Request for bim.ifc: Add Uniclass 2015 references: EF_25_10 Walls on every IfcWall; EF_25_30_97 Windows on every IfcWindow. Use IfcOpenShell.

First a look at what the model holds.

```python
import ifcopenshell

model = ifcopenshell.open("bim.ifc")
print(model.schema)
print("classifications:", [c.Name for c in model.by_type("IfcClassification")])
for ifc_class in ("IfcDoor", "IfcRoof", "IfcStair", "IfcWall", "IfcWindow"):
    print(ifc_class, len(model.by_type(ifc_class)))
```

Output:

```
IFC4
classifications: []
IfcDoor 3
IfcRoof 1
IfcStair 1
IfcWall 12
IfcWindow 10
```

```python
import ifcopenshell
import ifcopenshell.api.classification

model = ifcopenshell.open("bim.ifc")

system = ifcopenshell.api.classification.add_classification(model, classification="Uniclass 2015")

codes = {
    "IfcWall": ("EF_25_10", "Walls"),
    "IfcWindow": ("EF_25_30_97", "Windows"),
}
for ifc_class, (code, name) in codes.items():
    products = model.by_type(ifc_class)
    ifcopenshell.api.classification.add_reference(
        model, products=products, classification=system, identification=code, name=name
    )
    print(code, len(products))

model.write("bim_v2.ifc")
```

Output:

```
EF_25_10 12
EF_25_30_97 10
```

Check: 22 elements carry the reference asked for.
